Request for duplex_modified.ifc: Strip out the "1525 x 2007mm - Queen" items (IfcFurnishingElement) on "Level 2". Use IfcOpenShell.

First a look at what the model holds.

```python
import ifcopenshell
import ifcopenshell.util.element

model = ifcopenshell.open("duplex_modified.ifc")
print(model.schema)
storey = next(s for s in model.by_type("IfcBuildingStorey") if s.Name == "Level 2")
furniture = [e for e in ifcopenshell.util.element.get_decomposition(storey) if e.is_a("IfcFurnishingElement")]
seen = {}
for e in furniture:
    element_type = ifcopenshell.util.element.get_type(e)
    name = element_type.Name if element_type not in (None, e) else None
    seen[name] = seen.get(name, 0) + 1
for name, count in sorted(seen.items(), key=str):
    print(count, "x", name)
```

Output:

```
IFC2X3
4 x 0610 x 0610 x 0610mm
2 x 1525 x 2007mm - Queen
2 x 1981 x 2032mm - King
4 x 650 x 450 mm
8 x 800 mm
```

```python
import ifcopenshell
import ifcopenshell.api.root
import ifcopenshell.util.element

model = ifcopenshell.open("duplex_modified.ifc")

storey = next(s for s in model.by_type("IfcBuildingStorey") if s.Name == "Level 2")
furniture = [e for e in ifcopenshell.util.element.get_decomposition(storey) if e.is_a("IfcFurnishingElement")]
targets = [e for e in furniture if (t := ifcopenshell.util.element.get_type(e)) not in (None, e) and t.Name == "1525 x 2007mm - Queen"]

for e in targets:
    ifcopenshell.api.root.remove_product(model, product=e)
print(len(targets), "removed")

model.write("duplex_modified_updated.ifc")
```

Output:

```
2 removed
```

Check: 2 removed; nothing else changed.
